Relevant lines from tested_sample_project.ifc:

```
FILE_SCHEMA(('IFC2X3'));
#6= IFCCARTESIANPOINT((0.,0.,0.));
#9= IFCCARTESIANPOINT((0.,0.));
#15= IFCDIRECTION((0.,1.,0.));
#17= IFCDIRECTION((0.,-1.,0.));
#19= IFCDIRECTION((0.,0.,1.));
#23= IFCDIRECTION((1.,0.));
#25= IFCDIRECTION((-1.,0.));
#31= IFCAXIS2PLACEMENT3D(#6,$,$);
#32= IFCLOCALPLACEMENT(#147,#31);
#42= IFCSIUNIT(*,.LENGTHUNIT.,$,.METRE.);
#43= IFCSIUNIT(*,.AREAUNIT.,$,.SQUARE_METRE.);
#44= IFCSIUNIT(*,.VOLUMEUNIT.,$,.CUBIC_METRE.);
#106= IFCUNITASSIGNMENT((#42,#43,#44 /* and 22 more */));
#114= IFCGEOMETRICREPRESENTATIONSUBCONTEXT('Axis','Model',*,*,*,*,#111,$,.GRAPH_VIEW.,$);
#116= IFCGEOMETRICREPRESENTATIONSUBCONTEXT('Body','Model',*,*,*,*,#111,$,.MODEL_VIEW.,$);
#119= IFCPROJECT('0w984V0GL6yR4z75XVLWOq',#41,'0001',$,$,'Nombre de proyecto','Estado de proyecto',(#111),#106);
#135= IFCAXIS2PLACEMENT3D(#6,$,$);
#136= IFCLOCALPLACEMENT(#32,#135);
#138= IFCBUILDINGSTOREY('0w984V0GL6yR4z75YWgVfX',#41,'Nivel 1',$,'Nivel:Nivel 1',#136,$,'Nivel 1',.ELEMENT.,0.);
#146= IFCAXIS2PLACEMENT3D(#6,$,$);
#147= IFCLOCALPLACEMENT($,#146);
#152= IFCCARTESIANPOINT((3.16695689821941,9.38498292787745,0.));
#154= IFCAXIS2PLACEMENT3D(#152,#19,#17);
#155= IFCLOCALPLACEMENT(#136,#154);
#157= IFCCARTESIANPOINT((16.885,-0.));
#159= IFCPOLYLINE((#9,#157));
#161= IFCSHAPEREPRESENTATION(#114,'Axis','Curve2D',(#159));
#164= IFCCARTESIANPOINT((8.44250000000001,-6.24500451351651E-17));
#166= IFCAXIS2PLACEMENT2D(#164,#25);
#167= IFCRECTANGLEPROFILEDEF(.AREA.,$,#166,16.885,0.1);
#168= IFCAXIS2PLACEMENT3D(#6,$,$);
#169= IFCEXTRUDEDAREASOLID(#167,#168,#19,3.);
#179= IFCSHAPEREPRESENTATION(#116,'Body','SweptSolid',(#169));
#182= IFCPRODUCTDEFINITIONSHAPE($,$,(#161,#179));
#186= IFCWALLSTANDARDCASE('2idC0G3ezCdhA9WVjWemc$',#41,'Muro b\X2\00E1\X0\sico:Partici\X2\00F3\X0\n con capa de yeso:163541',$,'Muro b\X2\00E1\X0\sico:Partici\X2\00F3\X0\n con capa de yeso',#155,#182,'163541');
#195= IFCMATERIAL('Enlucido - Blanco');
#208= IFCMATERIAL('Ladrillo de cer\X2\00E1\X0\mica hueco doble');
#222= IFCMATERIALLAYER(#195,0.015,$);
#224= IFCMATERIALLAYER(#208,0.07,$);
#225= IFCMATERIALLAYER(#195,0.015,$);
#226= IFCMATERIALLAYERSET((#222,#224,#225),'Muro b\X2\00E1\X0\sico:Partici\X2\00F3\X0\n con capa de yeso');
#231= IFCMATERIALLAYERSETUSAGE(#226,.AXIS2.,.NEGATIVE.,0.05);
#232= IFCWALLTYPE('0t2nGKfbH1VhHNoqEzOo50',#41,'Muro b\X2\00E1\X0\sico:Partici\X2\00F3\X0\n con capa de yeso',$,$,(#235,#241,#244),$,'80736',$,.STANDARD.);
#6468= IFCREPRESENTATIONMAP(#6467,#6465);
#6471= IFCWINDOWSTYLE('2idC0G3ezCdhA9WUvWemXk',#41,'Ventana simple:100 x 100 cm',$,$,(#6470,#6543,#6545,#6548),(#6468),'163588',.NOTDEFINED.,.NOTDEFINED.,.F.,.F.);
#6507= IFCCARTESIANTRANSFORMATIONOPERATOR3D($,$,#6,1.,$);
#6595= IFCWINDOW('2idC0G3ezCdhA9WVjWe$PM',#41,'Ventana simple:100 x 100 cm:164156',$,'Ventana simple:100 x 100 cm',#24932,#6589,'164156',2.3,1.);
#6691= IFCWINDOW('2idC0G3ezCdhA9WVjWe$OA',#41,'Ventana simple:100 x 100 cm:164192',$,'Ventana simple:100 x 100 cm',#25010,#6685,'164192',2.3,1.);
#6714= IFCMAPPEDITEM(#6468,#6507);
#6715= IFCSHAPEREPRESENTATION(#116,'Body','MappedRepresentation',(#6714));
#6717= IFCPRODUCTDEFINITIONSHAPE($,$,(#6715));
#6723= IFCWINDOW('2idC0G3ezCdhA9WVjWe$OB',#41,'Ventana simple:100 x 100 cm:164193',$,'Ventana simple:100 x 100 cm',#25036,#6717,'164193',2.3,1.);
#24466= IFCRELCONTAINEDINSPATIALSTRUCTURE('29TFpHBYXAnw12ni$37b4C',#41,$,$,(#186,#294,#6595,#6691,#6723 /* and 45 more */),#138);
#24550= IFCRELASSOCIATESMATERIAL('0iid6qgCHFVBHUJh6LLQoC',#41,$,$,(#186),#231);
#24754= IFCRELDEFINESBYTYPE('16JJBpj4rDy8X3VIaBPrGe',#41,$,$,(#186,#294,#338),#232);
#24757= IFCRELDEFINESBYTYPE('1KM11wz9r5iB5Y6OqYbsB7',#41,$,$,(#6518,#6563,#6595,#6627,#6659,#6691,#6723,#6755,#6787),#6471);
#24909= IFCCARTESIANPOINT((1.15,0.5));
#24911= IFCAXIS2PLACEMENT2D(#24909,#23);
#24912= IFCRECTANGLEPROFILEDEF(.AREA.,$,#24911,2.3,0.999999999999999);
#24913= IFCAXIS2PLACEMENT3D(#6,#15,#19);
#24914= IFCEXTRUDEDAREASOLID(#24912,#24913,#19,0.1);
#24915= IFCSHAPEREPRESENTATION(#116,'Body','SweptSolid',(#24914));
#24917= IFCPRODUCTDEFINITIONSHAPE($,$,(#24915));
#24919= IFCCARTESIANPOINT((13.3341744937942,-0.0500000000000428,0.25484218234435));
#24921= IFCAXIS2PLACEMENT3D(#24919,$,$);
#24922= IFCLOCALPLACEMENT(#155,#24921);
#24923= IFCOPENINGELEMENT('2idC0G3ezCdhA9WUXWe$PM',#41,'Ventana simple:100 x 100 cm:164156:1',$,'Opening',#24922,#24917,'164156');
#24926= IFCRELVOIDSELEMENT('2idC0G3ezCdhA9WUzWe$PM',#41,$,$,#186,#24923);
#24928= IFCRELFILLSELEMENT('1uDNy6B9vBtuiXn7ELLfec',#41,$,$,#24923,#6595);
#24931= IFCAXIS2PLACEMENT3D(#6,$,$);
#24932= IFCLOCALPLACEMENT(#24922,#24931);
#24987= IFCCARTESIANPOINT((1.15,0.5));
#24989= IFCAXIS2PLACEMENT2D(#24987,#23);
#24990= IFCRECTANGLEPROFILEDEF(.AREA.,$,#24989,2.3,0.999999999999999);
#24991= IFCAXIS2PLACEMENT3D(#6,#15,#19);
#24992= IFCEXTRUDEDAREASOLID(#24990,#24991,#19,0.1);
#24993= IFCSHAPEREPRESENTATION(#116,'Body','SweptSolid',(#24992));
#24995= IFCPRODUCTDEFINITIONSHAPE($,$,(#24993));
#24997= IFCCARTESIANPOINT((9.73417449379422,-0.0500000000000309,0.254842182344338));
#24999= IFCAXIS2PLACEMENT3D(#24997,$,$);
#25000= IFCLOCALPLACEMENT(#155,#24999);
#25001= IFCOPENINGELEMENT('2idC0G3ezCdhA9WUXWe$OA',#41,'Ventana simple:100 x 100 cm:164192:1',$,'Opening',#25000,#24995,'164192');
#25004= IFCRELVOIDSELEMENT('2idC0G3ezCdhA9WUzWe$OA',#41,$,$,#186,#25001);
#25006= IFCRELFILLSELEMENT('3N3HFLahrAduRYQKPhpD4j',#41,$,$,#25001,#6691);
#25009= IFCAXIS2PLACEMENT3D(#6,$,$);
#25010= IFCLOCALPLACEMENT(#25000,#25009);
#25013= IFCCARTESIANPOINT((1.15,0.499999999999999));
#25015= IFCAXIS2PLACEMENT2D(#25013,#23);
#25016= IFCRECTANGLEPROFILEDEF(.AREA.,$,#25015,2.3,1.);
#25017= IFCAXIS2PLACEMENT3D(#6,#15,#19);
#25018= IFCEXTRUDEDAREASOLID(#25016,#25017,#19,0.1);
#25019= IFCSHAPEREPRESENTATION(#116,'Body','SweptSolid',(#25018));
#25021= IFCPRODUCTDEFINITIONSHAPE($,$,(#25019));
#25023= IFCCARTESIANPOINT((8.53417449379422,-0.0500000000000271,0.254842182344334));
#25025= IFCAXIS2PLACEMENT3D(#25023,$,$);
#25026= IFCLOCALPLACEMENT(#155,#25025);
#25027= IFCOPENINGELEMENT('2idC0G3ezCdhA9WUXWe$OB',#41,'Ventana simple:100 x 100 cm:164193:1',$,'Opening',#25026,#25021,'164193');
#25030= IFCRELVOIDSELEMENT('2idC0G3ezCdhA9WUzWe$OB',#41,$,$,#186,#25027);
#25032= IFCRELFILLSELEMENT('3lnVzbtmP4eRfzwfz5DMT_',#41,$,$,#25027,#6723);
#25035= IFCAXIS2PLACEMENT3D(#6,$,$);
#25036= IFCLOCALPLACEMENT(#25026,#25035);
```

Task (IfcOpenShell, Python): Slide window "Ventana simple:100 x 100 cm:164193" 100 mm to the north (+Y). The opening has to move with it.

```python
import ifcopenshell
import ifcopenshell.api.geometry
import ifcopenshell.util.placement
import ifcopenshell.util.unit

model = ifcopenshell.open("tested_sample_project.ifc")
unit_scale = ifcopenshell.util.unit.calculate_unit_scale(model)

window = model.by_id(6723)
opening = window.FillsVoids[0].RelatingOpeningElement
wall = opening.VoidsElements[0].RelatingBuildingElement

wall_matrix = ifcopenshell.util.placement.get_local_placement(wall.ObjectPlacement)
shift = wall_matrix[:3, 0] * -0.1 / unit_scale
before = ifcopenshell.util.placement.get_local_placement(window.ObjectPlacement)[:3, 3].copy()

# The window is placed relative to its opening, so it follows when the opening moves.
matrix = ifcopenshell.util.placement.get_local_placement(opening.ObjectPlacement)
matrix[:3, 3] += shift
ifcopenshell.api.geometry.edit_object_placement(
    model, product=opening, matrix=matrix, is_si=False, should_transform_children=True
)

after = ifcopenshell.util.placement.get_local_placement(window.ObjectPlacement)[:3, 3]
print("window moved by", (after - before).round(3) + 0.0)

model.write("tested_sample_project-out.ifc")
```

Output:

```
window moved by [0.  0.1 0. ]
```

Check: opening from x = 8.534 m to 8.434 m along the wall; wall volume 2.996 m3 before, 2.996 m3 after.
